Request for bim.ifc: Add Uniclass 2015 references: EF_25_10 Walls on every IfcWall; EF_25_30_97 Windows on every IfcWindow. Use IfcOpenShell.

First a look at what the model holds.

```python
import ifcopenshell

model = ifcopenshell.open("bim.ifc")
print(model.schema)
print("classifications:", [c.Name for c in model.by_type("IfcClassification")])
for ifc_class in ("IfcDoor", "IfcRoof", "IfcStair", "IfcWall", "IfcWindow"):
    print(ifc_class, len(model.by_type(ifc_class)))
```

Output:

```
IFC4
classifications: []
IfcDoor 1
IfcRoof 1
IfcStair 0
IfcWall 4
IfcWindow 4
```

```python
import ifcopenshell
import ifcopenshell.api.classification

model = ifcopenshell.open("bim.ifc")

system = ifcopenshell.api.classification.add_classification(model, classification="Uniclass 2015")

codes = {
    "IfcWall": ("EF_25_10", "Walls"),
    "IfcWindow": ("EF_25_30_97", "Windows"),
}
for ifc_class, (code, name) in codes.items():
    products = model.by_type(ifc_class)
    ifcopenshell.api.classification.add_reference(
        model, products=products, classification=system, identification=code, name=name
    )
    print(code, len(products))

model.write("bim_updated.ifc")
```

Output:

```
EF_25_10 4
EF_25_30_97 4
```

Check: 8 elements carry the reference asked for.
